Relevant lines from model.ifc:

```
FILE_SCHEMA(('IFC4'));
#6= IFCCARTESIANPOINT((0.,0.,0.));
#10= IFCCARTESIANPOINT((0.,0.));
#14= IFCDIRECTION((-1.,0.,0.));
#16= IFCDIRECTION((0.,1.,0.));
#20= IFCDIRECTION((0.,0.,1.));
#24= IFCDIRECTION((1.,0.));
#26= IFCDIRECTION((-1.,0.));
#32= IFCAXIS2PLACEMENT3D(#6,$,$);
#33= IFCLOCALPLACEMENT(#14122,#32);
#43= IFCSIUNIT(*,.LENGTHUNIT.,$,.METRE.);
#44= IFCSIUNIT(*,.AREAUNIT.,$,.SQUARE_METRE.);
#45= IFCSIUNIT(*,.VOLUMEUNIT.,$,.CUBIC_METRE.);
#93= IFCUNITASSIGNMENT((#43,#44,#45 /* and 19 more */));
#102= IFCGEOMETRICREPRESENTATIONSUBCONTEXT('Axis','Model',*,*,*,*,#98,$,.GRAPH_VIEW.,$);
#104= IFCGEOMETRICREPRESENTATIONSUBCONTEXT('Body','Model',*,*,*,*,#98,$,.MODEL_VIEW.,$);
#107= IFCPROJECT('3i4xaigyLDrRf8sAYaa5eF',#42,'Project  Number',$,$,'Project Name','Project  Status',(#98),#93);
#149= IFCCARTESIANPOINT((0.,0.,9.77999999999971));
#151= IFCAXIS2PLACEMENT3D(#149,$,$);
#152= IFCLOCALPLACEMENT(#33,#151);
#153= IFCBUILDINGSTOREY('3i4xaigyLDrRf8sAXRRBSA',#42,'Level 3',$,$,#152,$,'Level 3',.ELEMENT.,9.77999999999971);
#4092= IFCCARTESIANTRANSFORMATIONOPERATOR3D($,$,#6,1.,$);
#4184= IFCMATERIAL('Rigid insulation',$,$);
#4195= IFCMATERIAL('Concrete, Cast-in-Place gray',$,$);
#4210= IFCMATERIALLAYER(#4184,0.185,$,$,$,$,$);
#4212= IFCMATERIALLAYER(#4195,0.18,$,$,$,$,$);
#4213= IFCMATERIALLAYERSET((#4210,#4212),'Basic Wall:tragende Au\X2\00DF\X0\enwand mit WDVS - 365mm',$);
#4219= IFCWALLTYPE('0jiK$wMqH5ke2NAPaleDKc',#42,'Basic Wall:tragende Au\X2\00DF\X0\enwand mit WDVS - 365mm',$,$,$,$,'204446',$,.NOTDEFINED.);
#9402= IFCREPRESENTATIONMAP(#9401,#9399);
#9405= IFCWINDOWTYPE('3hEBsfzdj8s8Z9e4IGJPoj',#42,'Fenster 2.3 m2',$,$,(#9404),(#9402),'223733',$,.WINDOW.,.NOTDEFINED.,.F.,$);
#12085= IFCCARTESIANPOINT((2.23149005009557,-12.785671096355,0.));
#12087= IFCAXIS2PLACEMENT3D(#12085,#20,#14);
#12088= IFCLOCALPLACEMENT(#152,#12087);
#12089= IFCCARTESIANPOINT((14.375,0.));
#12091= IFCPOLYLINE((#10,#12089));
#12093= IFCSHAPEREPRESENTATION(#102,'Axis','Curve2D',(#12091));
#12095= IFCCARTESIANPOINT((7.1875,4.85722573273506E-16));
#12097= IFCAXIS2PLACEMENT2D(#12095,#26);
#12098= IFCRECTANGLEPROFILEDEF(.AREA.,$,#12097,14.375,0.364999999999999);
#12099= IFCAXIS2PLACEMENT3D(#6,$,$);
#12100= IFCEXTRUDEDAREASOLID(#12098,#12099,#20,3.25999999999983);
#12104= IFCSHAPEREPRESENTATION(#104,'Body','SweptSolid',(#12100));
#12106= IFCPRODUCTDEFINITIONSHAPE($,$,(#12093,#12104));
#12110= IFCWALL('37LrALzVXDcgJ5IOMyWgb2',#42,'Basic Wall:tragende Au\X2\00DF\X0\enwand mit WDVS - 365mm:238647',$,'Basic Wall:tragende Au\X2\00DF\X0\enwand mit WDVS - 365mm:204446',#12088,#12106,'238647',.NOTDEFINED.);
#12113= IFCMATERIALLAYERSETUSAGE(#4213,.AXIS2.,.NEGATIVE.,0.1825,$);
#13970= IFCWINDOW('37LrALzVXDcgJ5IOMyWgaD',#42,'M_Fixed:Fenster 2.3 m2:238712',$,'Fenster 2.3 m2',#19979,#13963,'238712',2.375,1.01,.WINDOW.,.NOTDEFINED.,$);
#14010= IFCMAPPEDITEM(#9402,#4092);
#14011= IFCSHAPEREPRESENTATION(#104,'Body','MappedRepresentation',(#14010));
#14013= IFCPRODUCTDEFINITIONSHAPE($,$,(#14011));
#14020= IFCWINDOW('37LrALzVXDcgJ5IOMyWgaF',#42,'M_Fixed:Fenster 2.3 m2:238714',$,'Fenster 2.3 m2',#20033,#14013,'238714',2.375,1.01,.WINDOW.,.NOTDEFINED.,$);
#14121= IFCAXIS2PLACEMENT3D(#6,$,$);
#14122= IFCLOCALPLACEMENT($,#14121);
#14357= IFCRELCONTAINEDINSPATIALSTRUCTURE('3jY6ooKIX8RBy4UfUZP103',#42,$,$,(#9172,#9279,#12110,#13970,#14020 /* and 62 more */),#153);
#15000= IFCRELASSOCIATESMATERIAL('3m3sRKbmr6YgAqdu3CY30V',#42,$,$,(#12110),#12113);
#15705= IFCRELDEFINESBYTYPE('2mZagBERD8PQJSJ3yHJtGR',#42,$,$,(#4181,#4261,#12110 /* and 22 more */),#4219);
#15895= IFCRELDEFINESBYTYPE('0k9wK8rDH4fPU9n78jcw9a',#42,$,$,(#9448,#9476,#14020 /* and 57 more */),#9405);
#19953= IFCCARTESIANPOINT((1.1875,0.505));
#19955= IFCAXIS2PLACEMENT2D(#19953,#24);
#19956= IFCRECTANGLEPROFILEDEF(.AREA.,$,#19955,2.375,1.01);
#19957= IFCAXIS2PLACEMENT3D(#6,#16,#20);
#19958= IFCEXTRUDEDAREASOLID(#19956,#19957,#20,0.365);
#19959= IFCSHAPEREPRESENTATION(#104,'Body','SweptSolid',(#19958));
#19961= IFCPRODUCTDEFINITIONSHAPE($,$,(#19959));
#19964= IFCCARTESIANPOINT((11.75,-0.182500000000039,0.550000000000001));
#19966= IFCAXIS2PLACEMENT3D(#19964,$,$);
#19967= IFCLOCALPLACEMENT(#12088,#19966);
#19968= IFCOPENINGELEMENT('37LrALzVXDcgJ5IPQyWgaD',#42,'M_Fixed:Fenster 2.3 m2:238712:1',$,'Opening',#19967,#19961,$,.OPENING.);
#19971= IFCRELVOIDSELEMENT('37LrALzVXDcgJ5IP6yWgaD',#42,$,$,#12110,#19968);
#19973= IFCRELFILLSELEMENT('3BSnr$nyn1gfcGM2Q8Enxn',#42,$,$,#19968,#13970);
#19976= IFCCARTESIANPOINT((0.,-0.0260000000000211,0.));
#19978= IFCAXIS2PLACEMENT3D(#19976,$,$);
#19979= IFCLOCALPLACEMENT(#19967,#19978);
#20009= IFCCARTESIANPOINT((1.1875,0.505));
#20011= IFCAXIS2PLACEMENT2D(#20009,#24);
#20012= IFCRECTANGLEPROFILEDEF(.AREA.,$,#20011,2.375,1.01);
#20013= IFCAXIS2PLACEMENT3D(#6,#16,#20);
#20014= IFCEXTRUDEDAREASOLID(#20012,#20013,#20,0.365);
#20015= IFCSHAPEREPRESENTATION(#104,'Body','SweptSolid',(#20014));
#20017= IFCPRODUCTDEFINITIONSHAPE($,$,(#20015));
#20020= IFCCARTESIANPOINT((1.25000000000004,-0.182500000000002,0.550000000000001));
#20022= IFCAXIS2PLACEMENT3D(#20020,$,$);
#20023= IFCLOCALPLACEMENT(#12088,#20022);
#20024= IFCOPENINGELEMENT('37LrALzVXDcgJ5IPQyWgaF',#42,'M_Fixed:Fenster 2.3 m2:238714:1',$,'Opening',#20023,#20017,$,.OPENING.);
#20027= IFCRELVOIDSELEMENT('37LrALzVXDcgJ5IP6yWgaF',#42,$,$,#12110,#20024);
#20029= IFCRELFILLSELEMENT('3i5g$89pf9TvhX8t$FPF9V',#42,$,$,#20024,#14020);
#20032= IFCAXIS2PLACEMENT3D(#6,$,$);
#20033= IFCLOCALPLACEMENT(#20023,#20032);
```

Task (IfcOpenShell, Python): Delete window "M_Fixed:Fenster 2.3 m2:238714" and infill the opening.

```python
import ifcopenshell
import ifcopenshell.api.feature
import ifcopenshell.api.root
import ifcopenshell.geom
import ifcopenshell.util.shape

model = ifcopenshell.open("model.ifc")
settings = ifcopenshell.geom.settings()


def volume(element):
    """Net volume in cubic metres, openings subtracted."""
    shape = ifcopenshell.geom.create_shape(settings, element)
    return ifcopenshell.util.shape.get_volume(shape.geometry)


window = model.by_id(14020)
opening = window.FillsVoids[0].RelatingOpeningElement
wall = opening.VoidsElements[0].RelatingBuildingElement
before = volume(wall)

ifcopenshell.api.root.remove_product(model, product=window)
ifcopenshell.api.feature.remove_feature(model, feature=opening)

after = volume(wall)

print(f"wall volume {before:.3f} -> {after:.3f} m3")

model.write("model_v2.ifc")
```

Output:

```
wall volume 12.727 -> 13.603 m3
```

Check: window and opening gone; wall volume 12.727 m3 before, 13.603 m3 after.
